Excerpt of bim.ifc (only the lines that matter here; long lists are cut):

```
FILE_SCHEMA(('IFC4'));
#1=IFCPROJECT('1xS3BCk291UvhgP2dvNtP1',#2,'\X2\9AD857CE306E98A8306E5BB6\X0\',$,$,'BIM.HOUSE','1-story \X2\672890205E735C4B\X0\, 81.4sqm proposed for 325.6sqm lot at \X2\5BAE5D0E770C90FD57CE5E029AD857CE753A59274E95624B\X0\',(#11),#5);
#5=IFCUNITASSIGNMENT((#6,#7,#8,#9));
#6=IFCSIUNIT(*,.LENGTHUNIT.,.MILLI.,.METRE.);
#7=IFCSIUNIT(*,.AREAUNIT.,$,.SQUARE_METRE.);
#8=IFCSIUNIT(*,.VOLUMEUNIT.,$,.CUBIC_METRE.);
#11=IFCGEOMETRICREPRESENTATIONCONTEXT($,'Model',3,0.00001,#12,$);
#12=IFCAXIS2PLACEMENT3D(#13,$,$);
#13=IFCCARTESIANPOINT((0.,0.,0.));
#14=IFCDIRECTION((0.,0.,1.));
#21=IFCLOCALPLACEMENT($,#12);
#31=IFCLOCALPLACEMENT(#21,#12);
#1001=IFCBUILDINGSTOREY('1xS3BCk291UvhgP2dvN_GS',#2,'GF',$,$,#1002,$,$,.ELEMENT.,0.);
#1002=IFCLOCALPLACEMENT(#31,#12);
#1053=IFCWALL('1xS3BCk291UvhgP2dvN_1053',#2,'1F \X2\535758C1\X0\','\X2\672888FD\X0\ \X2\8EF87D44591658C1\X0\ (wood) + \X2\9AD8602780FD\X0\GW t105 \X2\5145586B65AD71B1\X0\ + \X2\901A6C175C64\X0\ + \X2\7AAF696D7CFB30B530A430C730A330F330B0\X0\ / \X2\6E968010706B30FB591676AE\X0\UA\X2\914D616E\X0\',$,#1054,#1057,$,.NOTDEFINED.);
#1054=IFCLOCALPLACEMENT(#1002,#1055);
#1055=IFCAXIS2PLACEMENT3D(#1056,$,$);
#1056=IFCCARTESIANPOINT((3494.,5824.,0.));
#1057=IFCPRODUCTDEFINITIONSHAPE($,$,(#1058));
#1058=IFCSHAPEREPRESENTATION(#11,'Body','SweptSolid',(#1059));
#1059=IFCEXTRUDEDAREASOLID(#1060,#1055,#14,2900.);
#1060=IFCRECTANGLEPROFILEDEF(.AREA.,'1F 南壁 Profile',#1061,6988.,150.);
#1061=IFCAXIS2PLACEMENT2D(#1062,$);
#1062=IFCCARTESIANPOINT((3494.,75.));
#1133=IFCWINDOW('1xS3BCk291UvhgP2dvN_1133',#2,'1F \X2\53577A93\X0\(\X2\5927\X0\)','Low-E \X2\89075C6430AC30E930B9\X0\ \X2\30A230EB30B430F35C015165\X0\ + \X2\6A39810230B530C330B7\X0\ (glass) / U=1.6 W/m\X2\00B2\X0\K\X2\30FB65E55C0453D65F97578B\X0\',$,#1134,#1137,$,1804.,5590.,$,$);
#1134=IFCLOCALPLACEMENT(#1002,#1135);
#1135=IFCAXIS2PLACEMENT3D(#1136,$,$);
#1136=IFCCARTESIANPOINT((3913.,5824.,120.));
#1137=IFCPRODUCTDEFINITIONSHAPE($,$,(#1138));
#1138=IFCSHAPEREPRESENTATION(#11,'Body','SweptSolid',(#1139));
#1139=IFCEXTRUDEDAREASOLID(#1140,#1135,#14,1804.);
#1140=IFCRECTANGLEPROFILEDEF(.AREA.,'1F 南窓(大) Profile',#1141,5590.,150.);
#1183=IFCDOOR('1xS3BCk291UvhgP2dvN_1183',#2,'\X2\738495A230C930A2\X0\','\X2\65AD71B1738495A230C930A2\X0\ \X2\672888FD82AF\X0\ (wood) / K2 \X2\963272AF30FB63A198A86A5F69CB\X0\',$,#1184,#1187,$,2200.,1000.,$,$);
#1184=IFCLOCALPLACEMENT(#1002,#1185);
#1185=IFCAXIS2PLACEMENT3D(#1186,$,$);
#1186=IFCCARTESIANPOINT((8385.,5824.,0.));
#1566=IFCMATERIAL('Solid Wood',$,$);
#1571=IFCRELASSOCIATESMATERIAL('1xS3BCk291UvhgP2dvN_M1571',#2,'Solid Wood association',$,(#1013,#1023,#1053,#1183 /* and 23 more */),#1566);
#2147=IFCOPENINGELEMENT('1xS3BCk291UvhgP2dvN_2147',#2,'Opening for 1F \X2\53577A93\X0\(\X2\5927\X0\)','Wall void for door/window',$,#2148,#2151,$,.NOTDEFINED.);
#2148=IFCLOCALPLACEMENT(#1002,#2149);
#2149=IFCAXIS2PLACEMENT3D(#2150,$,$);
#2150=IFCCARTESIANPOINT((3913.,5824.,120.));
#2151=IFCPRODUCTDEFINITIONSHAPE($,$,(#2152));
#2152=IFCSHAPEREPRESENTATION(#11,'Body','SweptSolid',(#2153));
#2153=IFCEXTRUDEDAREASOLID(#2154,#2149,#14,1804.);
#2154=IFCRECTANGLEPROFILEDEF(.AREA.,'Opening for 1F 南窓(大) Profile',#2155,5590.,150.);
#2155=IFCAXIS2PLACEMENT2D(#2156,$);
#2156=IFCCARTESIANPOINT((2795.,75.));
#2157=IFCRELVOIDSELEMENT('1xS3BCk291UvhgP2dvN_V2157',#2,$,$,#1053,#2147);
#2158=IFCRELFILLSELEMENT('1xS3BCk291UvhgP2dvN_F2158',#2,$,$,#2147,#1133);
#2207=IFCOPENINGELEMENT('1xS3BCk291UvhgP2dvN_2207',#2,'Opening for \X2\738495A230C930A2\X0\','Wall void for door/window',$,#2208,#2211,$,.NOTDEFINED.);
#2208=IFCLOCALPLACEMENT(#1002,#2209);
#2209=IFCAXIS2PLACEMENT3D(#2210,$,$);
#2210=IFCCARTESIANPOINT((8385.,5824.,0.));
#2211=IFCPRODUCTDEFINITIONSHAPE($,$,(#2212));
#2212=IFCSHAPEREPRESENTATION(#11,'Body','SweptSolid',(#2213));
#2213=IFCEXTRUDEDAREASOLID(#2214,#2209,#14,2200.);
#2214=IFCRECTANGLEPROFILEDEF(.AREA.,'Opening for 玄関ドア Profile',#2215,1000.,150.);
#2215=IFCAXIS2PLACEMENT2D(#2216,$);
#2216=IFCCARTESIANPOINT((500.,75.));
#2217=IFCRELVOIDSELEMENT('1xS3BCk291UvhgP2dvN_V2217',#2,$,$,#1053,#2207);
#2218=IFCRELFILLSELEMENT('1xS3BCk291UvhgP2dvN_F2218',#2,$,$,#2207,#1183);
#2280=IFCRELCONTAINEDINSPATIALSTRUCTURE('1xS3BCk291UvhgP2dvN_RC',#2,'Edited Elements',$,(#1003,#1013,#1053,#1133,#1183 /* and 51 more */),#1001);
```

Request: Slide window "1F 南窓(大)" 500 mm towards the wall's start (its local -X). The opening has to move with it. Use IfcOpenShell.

```python
import ifcopenshell
import ifcopenshell.api.geometry
import ifcopenshell.util.placement
import ifcopenshell.util.unit

model = ifcopenshell.open("bim.ifc")
unit_scale = ifcopenshell.util.unit.calculate_unit_scale(model)

window = model.by_guid("1xS3BCk291UvhgP2dvN_1133")
opening = window.FillsVoids[0].RelatingOpeningElement
wall = opening.VoidsElements[0].RelatingBuildingElement

wall_matrix = ifcopenshell.util.placement.get_local_placement(wall.ObjectPlacement)
shift = wall_matrix[:3, 0] * -0.5 / unit_scale
before = ifcopenshell.util.placement.get_local_placement(window.ObjectPlacement)[:3, 3].copy()

# The window is not placed relative to its opening, so move both.
for product in (opening, window):
    matrix = ifcopenshell.util.placement.get_local_placement(product.ObjectPlacement)
    matrix[:3, 3] += shift
    ifcopenshell.api.geometry.edit_object_placement(model, product=product, matrix=matrix, is_si=False)

after = ifcopenshell.util.placement.get_local_placement(window.ObjectPlacement)[:3, 3]
print("window moved by", (after - before).round(3) + 0.0)

model.write("bim-out.ifc")
```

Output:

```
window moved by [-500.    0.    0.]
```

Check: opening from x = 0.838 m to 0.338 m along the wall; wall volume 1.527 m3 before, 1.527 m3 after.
